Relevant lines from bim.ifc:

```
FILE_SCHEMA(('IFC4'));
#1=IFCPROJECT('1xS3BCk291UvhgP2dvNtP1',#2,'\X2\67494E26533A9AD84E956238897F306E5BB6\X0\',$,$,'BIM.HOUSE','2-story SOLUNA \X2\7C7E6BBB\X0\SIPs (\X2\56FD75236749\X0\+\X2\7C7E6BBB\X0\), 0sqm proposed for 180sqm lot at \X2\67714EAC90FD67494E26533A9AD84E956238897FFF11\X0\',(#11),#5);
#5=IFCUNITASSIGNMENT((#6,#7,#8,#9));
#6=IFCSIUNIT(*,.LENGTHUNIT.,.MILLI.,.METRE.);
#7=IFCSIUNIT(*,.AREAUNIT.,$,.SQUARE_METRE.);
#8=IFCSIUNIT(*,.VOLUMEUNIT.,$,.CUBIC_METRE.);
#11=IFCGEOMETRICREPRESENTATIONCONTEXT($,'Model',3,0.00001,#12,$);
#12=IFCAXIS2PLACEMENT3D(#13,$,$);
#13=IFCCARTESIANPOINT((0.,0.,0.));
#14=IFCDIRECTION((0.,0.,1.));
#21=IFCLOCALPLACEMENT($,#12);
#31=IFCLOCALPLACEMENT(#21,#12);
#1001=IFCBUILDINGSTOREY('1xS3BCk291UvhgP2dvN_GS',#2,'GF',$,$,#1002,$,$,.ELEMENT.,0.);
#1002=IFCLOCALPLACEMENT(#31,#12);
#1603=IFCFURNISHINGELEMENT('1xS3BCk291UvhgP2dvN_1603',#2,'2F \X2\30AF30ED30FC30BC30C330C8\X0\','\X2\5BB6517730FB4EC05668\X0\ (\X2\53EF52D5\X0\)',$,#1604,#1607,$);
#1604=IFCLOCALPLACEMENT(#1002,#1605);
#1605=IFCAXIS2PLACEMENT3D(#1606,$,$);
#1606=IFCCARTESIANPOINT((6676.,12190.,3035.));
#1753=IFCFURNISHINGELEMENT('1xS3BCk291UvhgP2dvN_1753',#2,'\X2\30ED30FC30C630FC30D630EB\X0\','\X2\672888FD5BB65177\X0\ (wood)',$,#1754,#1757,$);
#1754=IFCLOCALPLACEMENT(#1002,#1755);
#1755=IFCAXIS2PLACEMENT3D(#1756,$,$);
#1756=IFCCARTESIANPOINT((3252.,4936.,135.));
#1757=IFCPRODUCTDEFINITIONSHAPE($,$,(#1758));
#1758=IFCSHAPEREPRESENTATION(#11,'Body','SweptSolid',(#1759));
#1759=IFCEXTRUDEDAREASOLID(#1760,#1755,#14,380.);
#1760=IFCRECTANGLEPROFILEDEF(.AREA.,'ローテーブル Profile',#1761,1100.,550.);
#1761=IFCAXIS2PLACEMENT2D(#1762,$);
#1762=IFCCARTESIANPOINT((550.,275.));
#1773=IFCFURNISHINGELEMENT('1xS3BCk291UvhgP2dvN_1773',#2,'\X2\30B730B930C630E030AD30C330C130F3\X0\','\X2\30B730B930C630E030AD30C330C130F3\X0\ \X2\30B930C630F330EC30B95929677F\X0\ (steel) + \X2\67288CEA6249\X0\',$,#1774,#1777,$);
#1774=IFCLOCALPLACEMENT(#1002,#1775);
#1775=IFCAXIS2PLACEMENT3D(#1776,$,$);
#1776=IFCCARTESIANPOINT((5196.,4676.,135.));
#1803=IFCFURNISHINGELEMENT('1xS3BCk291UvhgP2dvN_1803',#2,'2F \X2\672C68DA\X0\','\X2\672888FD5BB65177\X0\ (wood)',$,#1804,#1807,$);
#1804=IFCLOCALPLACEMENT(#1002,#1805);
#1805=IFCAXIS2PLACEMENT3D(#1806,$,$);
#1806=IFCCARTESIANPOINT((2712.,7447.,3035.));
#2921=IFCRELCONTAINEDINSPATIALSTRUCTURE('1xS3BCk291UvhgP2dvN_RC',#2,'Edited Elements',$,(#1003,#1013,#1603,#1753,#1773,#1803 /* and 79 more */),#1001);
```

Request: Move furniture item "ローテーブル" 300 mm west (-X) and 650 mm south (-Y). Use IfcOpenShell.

```python
import ifcopenshell
import ifcopenshell.api.geometry
import ifcopenshell.util.placement
import ifcopenshell.util.unit

model = ifcopenshell.open("bim.ifc")
unit_scale = ifcopenshell.util.unit.calculate_unit_scale(model)

item = model.by_guid("1xS3BCk291UvhgP2dvN_1753")
matrix = ifcopenshell.util.placement.get_local_placement(item.ObjectPlacement)
matrix[0, 3] -= 0.3 / unit_scale
matrix[1, 3] -= 0.65 / unit_scale
ifcopenshell.api.geometry.edit_object_placement(model, product=item, matrix=matrix, is_si=False)

print(ifcopenshell.util.placement.get_local_placement(item.ObjectPlacement).round(3) + 0.0)

model.write("bim_edited.ifc")
```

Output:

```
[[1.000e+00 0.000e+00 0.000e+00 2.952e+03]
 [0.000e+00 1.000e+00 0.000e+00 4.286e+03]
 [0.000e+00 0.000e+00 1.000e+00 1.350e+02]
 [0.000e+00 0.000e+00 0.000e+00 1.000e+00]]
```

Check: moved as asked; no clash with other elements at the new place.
